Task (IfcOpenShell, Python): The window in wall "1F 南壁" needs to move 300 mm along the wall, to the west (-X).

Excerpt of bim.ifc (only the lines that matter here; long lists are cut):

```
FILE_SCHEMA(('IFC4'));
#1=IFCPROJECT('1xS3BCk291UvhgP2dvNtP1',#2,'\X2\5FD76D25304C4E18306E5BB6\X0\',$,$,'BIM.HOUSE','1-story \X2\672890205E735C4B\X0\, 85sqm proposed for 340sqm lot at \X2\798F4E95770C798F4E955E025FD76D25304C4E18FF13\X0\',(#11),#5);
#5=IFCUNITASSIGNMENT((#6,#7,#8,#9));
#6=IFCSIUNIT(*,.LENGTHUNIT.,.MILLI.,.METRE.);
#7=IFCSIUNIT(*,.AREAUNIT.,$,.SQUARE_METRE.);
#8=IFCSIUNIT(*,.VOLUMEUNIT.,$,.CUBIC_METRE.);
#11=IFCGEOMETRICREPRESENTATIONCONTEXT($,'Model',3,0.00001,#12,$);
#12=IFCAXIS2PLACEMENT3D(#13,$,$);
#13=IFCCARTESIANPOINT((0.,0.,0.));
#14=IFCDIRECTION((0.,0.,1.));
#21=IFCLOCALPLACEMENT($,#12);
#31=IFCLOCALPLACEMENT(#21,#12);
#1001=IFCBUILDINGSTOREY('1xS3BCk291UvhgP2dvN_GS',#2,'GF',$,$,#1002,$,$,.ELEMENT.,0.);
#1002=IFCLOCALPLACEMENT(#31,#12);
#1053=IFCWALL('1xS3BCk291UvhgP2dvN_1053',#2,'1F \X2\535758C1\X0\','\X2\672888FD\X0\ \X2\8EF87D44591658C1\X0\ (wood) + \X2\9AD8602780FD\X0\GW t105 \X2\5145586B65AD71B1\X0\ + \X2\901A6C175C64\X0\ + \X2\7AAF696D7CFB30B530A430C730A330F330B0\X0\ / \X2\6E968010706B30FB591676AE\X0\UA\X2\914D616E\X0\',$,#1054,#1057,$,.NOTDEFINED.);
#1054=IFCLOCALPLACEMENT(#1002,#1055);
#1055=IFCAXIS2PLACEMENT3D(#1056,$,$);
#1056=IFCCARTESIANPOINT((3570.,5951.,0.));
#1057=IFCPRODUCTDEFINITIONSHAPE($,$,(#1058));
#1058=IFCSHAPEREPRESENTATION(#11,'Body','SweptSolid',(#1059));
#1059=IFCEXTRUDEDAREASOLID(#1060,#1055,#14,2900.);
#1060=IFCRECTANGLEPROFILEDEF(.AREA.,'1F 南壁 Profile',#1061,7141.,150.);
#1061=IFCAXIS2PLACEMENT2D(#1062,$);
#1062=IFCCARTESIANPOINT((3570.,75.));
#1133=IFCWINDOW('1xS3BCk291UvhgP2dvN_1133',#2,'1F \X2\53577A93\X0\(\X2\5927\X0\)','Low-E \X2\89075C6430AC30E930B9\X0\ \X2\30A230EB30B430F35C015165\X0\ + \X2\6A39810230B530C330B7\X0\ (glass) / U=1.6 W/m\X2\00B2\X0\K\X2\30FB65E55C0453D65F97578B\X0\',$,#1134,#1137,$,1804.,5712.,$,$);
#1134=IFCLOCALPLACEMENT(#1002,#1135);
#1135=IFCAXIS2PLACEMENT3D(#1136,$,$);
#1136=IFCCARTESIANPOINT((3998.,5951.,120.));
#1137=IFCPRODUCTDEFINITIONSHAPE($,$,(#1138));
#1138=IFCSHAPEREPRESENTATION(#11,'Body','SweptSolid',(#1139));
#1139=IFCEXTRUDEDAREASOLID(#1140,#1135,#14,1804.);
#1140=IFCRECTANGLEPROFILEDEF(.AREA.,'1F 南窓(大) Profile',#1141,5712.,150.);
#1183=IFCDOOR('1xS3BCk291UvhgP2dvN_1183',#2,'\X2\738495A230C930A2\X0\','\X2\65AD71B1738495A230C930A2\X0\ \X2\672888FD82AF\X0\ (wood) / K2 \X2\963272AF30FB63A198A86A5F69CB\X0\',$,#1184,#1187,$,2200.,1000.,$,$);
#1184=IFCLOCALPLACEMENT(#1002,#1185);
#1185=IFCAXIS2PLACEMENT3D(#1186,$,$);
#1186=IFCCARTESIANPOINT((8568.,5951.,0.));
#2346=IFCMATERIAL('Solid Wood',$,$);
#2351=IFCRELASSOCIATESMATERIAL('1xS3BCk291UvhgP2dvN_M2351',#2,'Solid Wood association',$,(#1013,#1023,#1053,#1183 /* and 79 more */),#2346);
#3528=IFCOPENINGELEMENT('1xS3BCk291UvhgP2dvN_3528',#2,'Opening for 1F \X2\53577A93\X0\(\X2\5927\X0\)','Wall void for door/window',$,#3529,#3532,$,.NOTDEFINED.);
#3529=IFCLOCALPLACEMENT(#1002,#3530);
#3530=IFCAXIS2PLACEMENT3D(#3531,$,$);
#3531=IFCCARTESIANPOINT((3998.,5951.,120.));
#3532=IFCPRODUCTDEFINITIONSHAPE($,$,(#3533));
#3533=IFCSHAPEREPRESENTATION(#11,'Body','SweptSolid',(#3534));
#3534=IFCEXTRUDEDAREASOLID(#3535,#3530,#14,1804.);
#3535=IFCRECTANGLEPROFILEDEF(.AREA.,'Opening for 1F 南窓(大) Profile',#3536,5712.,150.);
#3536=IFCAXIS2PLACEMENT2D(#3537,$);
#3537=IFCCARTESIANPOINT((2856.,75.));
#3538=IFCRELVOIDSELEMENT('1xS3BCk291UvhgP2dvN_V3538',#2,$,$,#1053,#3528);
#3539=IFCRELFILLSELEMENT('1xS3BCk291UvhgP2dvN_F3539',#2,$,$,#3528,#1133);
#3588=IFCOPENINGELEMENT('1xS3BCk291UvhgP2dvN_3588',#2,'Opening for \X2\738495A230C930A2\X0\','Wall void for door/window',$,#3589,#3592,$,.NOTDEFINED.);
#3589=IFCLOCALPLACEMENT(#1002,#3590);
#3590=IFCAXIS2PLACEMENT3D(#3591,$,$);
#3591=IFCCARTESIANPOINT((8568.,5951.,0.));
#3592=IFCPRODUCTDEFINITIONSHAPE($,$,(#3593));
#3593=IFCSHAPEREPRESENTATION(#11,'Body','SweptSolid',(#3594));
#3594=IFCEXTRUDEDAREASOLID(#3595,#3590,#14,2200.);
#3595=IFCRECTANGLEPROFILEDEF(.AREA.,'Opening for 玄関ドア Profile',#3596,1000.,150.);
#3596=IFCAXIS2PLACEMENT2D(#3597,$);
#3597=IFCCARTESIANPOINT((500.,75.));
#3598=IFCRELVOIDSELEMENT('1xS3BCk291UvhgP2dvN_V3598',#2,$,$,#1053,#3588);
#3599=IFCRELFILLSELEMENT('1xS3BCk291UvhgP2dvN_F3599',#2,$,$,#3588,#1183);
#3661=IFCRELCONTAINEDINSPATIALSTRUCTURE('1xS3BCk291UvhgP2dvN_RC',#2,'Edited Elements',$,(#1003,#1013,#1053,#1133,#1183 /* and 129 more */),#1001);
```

```python
import ifcopenshell
import ifcopenshell.api.geometry
import ifcopenshell.util.placement
import ifcopenshell.util.unit

model = ifcopenshell.open("bim.ifc")
unit_scale = ifcopenshell.util.unit.calculate_unit_scale(model)

window = model.by_guid("1xS3BCk291UvhgP2dvN_1133")
opening = window.FillsVoids[0].RelatingOpeningElement
wall = opening.VoidsElements[0].RelatingBuildingElement

wall_matrix = ifcopenshell.util.placement.get_local_placement(wall.ObjectPlacement)
shift = wall_matrix[:3, 0] * -0.3 / unit_scale
before = ifcopenshell.util.placement.get_local_placement(window.ObjectPlacement)[:3, 3].copy()

# The window is not placed relative to its opening, so move both.
for product in (opening, window):
    matrix = ifcopenshell.util.placement.get_local_placement(product.ObjectPlacement)
    matrix[:3, 3] += shift
    ifcopenshell.api.geometry.edit_object_placement(model, product=product, matrix=matrix, is_si=False)

after = ifcopenshell.util.placement.get_local_placement(window.ObjectPlacement)[:3, 3]
print("window moved by", (after - before).round(3) + 0.0)

model.write("bim_edited.ifc")
```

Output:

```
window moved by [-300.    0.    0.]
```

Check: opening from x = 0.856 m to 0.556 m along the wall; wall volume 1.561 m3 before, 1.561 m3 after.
